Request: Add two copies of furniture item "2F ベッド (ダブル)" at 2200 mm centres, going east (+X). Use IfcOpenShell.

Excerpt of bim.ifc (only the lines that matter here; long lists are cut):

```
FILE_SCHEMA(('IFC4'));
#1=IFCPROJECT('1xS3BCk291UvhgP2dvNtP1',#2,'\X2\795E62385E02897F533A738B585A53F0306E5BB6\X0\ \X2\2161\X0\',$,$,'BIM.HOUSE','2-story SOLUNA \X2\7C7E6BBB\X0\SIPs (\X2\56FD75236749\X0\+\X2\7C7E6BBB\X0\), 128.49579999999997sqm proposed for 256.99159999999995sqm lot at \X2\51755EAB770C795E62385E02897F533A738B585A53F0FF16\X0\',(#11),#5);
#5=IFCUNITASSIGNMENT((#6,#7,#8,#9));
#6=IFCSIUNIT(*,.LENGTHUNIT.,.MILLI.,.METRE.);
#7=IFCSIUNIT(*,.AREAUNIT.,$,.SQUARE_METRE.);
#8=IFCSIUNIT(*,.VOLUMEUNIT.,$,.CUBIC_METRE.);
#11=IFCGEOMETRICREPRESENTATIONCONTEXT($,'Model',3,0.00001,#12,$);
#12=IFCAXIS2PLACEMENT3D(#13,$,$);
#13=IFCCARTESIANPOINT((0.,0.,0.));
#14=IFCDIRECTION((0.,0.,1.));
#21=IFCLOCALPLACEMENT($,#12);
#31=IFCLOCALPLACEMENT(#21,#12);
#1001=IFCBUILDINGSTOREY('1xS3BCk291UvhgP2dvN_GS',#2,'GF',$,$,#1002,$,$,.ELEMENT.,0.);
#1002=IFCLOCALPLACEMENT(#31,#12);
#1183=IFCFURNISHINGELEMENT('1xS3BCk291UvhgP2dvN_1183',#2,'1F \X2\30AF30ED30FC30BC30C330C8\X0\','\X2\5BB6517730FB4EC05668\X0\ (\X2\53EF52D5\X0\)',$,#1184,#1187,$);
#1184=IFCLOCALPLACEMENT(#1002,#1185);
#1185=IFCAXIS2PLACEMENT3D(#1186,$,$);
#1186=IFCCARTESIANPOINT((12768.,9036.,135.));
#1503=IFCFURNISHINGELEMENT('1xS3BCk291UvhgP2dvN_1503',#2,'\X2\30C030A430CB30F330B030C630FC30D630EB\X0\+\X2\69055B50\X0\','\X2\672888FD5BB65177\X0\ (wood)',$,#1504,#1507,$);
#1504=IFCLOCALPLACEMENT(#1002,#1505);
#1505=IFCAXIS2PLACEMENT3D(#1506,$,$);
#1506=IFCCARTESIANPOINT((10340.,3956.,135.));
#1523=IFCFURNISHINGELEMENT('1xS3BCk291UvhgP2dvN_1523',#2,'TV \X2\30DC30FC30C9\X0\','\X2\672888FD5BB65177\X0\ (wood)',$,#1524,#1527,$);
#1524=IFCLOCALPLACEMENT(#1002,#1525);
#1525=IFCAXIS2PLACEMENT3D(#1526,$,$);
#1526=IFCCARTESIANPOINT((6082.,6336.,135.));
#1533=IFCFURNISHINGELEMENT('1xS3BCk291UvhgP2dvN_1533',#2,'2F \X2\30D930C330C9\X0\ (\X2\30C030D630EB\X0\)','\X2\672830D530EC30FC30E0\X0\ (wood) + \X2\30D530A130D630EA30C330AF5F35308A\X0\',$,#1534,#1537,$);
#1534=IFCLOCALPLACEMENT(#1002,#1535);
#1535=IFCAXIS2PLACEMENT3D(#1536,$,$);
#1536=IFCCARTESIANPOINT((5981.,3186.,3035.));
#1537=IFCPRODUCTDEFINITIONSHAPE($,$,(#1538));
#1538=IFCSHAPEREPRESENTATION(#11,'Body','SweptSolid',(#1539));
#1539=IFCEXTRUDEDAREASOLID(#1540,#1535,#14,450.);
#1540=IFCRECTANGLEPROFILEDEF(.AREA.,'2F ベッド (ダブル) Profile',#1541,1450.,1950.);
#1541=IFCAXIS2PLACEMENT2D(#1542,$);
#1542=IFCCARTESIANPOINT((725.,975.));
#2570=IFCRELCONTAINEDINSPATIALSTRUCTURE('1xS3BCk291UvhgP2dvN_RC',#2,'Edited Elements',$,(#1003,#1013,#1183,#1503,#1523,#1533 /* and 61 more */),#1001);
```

```python
import numpy as np
import ifcopenshell
import ifcopenshell.api.geometry
import ifcopenshell.api.root
import ifcopenshell.util.element
import ifcopenshell.util.placement
import ifcopenshell.util.unit

model = ifcopenshell.open("bim.ifc")
unit_scale = ifcopenshell.util.unit.calculate_unit_scale(model)


def reuse_history(source, copy):
    """copy_class also copies each property set's owner history, people and application; keep the originals."""
    for rel in copy.IsDefinedBy:
        if rel.is_a("IfcRelDefinesByProperties") and (history := rel.RelatingPropertyDefinition.OwnerHistory):
            rel.RelatingPropertyDefinition.OwnerHistory = source.OwnerHistory
            ifcopenshell.util.element.remove_deep2(model, history)


source = model.by_guid("1xS3BCk291UvhgP2dvN_1533")
base = ifcopenshell.util.placement.get_local_placement(source.ObjectPlacement)
step = np.array([1.0, 0.0, 0.0]) * 2.2 / unit_scale

for i in range(1, 3):
    copy = ifcopenshell.api.root.copy_class(model, product=source)
    copy.Representation = ifcopenshell.util.element.copy_deep(
        model, source.Representation, exclude=["IfcGeometricRepresentationContext", "IfcRepresentationMap"]
    )
    reuse_history(source, copy)
    matrix = base.copy()
    matrix[:3, 3] += i * step
    print("added at", matrix[:3, 3].round(3) + 0.0)
    ifcopenshell.api.geometry.edit_object_placement(model, product=copy, matrix=matrix, is_si=False)

model.write("bim_rev.ifc")
```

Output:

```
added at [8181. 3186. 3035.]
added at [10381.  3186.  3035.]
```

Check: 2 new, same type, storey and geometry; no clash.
